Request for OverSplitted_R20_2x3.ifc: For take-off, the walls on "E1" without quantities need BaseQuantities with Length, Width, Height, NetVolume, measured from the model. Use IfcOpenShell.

First a look at what the model holds.

```python
import ifcopenshell
import ifcopenshell.util.element
import ifcopenshell.util.unit

model = ifcopenshell.open("OverSplitted_R20_2x3.ifc")
print(model.schema)
for unit_type in ("LENGTHUNIT", "AREAUNIT", "VOLUMEUNIT"):
    print(unit_type, ifcopenshell.util.unit.calculate_unit_scale(model, unit_type))
storey = next(s for s in model.by_type("IfcBuildingStorey") if s.Name == "E1")
walls = [e for e in ifcopenshell.util.element.get_decomposition(storey) if e.is_a("IfcWall")]
for e in sorted(walls, key=lambda e: e.id()):
    print(e.id(), e.is_a(), e.Name, list(ifcopenshell.util.element.get_psets(e, qtos_only=True)), sep=" | ")
```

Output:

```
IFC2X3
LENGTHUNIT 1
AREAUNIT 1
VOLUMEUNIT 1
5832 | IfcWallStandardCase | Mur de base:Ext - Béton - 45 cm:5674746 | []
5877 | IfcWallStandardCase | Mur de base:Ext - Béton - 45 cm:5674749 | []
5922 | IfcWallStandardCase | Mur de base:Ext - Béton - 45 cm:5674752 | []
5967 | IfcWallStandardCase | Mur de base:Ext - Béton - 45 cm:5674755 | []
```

```python
import ifcopenshell
import ifcopenshell.api.pset
import ifcopenshell.geom
import ifcopenshell.util.element
import ifcopenshell.util.shape
import ifcopenshell.util.unit

model = ifcopenshell.open("OverSplitted_R20_2x3.ifc")
unit_scale = ifcopenshell.util.unit.calculate_unit_scale(model)
volume_scale = ifcopenshell.util.unit.calculate_unit_scale(model, "VOLUMEUNIT")
settings = ifcopenshell.geom.settings()

storey = next(s for s in model.by_type("IfcBuildingStorey") if s.Name == "E1")
walls = [e for e in ifcopenshell.util.element.get_decomposition(storey) if e.is_a("IfcWall")]

for e in sorted(walls, key=lambda e: e.id()):
    if ifcopenshell.util.element.get_psets(e, qtos_only=True, should_inherit=False):
        continue
    # Geometry comes back in metres, in the element's own axes.
    shape = ifcopenshell.geom.create_shape(settings, e)
    values = {
        "Length": ifcopenshell.util.shape.get_x(shape.geometry) / unit_scale,
        "Width": ifcopenshell.util.shape.get_y(shape.geometry) / unit_scale,
        "Height": ifcopenshell.util.shape.get_z(shape.geometry) / unit_scale,
        "NetVolume": ifcopenshell.util.shape.get_volume(shape.geometry) / volume_scale,
    }
    qto = ifcopenshell.api.pset.add_qto(model, product=e, name="BaseQuantities")
    ifcopenshell.api.pset.edit_qto(model, qto=qto, properties=values)
    print(e.id(), {k: round(v, 3) for k, v in values.items()})

model.write("OverSplitted_R20_2x3_updated.ifc")
```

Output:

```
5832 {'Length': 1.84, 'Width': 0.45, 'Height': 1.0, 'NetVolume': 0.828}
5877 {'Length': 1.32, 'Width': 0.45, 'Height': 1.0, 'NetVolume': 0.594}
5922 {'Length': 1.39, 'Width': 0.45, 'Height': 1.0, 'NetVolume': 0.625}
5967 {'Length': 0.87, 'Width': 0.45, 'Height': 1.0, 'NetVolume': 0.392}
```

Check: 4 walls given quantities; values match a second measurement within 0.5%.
